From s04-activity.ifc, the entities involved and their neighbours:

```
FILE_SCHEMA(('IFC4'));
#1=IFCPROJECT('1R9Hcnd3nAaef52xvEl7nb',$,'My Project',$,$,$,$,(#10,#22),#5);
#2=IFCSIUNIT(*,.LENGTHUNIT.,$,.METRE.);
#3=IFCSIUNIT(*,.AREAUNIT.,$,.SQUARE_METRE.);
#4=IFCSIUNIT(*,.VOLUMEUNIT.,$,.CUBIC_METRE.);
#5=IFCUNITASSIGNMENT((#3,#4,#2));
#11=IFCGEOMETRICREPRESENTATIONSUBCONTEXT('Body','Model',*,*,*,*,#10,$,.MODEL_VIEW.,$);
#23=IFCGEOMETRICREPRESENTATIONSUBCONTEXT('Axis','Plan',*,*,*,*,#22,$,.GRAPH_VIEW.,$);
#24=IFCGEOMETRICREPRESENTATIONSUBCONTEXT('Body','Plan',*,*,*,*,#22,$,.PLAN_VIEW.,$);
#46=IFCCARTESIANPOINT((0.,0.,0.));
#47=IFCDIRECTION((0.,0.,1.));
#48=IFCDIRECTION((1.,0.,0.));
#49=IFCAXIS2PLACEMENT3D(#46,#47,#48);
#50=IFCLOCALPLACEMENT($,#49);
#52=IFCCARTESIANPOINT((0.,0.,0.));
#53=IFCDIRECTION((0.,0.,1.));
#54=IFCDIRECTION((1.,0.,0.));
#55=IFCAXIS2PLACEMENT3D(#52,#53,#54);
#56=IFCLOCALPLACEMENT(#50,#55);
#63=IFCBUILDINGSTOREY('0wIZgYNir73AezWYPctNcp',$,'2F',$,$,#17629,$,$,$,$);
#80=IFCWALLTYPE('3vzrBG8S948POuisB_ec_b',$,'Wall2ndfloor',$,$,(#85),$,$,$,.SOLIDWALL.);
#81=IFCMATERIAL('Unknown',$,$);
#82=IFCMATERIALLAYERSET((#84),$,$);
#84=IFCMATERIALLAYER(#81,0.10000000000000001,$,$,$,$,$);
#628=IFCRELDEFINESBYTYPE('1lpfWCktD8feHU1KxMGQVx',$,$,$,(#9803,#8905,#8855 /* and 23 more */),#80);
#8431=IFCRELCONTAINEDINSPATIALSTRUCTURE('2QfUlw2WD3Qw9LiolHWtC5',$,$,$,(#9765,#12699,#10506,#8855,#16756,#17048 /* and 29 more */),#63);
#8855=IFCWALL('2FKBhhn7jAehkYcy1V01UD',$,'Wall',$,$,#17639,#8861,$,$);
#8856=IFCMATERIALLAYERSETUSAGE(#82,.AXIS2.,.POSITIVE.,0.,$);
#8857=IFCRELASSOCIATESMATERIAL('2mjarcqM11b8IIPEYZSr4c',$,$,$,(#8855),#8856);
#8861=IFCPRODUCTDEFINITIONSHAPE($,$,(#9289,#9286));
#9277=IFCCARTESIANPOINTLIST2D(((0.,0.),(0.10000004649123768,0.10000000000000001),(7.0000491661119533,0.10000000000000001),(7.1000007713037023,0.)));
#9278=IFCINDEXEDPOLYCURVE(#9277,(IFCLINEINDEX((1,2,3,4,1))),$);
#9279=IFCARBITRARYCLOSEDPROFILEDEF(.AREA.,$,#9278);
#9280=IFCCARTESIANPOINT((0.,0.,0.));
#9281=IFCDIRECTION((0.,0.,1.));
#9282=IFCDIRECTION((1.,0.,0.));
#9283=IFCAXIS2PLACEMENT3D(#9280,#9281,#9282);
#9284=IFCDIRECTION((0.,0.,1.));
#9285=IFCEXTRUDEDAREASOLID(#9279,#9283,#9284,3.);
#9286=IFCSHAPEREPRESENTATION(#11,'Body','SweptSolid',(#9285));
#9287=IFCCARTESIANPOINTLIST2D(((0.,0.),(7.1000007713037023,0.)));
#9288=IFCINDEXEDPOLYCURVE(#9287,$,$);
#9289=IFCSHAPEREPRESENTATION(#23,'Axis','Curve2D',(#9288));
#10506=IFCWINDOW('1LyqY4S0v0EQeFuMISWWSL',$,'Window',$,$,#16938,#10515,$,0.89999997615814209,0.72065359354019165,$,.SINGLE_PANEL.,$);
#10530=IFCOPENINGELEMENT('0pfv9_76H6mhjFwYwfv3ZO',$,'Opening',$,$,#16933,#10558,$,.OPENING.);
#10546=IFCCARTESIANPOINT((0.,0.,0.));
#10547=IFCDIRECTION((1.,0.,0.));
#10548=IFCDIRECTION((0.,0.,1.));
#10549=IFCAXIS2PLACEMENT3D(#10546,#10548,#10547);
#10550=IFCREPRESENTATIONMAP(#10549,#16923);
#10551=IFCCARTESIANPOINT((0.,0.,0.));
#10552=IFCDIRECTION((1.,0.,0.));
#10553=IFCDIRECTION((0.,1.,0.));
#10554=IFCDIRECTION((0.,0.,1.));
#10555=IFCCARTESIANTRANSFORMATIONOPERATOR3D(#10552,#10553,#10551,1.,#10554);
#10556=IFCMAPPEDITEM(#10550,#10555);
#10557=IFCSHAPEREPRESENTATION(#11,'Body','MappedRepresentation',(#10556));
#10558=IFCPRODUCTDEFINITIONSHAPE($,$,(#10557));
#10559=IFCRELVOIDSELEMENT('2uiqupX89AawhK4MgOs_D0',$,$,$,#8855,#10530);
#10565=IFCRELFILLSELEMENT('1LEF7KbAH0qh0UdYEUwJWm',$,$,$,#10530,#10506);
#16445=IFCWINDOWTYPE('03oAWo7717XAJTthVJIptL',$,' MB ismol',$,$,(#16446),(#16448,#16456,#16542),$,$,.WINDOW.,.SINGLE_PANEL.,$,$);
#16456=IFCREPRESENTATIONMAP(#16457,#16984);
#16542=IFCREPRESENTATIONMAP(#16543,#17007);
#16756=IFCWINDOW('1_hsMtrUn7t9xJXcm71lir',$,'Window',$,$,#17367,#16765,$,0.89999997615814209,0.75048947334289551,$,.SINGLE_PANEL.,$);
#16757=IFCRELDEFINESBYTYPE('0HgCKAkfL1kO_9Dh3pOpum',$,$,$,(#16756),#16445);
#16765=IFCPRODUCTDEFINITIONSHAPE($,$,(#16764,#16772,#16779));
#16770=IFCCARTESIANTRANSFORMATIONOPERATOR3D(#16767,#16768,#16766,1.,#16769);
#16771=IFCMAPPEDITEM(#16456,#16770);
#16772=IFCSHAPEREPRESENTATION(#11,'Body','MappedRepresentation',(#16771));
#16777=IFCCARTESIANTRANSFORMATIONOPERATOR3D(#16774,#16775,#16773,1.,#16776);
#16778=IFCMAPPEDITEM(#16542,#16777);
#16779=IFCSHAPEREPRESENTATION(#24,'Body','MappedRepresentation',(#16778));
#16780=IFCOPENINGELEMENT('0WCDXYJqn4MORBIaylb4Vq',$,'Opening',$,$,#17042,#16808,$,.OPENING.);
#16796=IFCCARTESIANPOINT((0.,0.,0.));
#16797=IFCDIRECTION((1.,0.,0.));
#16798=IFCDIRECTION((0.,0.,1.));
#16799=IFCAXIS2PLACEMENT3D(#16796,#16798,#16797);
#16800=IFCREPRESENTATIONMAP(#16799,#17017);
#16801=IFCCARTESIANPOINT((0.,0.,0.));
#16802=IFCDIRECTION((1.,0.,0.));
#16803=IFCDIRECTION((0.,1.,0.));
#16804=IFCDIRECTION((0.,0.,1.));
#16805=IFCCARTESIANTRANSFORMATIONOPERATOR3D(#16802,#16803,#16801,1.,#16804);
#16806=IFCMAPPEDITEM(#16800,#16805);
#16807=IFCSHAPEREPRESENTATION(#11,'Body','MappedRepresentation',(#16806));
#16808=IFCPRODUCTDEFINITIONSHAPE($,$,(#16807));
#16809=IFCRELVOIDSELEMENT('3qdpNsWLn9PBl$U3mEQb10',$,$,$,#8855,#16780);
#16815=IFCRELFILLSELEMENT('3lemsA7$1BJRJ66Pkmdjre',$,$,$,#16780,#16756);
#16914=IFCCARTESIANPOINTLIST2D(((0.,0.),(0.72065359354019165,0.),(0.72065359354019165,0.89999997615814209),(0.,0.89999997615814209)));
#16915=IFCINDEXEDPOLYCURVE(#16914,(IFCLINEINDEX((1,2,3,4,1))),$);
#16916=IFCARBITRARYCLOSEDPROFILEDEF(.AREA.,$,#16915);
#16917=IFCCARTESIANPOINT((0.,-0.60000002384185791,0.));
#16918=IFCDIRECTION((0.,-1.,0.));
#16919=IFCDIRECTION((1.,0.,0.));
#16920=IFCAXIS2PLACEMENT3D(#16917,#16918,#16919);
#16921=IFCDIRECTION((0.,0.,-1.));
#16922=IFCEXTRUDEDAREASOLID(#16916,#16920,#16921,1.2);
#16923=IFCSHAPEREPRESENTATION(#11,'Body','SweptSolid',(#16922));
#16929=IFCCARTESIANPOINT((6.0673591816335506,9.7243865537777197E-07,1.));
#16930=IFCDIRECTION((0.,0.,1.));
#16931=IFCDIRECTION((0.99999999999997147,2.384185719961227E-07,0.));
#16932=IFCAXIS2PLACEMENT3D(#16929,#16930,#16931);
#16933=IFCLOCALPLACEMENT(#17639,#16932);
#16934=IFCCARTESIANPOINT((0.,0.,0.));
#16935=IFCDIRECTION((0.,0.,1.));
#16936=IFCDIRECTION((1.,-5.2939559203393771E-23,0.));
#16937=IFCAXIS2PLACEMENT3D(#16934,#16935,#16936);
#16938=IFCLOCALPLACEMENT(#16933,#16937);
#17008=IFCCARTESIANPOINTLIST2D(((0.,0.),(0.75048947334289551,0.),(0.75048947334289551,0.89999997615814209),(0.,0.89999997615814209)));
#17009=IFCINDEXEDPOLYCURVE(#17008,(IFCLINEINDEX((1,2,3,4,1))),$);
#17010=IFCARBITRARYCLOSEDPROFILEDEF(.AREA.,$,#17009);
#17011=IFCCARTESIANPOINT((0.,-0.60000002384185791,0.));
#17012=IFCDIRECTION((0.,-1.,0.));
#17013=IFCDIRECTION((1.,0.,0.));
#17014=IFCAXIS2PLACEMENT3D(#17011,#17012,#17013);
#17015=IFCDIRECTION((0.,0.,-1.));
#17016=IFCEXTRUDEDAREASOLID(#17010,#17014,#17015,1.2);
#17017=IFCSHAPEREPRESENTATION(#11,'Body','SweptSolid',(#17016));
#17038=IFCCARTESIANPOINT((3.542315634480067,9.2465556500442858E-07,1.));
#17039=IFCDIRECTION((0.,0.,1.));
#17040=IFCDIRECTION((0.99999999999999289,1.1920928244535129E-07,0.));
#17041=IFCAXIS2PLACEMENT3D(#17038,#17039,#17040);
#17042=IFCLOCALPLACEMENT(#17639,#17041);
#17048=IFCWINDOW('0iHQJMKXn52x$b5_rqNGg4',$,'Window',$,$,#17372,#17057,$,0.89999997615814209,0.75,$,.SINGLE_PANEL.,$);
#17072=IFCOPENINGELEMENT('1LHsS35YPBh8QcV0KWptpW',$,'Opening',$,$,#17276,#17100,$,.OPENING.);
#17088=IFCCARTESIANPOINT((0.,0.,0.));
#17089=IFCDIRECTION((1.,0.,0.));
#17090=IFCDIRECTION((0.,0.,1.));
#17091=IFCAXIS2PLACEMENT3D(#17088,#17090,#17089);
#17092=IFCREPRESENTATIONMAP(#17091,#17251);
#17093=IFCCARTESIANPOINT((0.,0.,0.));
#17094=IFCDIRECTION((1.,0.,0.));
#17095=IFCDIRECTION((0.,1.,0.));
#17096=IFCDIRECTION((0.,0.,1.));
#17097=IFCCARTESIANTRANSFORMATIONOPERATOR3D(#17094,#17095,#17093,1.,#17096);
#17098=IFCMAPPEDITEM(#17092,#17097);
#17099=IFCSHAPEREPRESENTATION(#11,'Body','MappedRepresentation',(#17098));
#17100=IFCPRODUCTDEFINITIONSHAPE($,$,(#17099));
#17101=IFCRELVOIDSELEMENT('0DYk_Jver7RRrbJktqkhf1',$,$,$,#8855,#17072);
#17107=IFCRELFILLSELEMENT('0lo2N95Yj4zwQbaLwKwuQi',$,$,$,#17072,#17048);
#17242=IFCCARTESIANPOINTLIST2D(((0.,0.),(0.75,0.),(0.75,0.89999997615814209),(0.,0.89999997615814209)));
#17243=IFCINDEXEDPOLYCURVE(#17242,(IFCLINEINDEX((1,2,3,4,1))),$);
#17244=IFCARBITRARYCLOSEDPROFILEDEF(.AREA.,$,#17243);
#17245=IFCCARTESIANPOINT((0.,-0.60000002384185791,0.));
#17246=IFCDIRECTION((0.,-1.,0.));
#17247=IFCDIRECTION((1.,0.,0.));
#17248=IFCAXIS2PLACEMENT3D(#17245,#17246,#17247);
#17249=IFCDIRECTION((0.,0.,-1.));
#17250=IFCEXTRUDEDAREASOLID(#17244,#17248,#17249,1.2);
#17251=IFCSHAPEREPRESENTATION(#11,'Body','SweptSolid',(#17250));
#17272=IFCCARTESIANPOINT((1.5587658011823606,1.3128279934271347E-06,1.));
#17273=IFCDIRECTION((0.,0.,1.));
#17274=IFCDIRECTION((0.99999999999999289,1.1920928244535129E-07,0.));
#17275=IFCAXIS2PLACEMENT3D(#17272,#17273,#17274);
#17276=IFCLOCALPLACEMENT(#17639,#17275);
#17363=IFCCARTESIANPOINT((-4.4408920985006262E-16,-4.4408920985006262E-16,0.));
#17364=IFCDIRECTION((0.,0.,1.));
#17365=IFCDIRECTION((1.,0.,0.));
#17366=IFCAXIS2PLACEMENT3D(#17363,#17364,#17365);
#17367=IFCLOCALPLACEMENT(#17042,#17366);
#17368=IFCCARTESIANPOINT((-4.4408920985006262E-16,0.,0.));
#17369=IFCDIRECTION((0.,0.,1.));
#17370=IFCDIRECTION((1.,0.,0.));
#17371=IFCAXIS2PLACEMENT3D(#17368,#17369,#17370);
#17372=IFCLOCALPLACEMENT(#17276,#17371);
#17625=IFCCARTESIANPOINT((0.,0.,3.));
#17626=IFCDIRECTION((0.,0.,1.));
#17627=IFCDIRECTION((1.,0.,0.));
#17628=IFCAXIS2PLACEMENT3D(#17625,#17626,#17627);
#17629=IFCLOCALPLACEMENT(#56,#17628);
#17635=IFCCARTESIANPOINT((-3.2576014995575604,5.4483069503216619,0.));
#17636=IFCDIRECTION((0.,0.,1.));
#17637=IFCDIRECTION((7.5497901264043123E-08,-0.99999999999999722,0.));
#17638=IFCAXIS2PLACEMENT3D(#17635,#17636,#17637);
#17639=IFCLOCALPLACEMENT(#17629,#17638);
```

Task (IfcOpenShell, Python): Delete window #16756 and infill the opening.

```python
import ifcopenshell
import ifcopenshell.api.feature
import ifcopenshell.api.root
import ifcopenshell.geom
import ifcopenshell.util.shape

model = ifcopenshell.open("s04-activity.ifc")
settings = ifcopenshell.geom.settings()


def volume(element):
    """Net volume in cubic metres, openings subtracted."""
    shape = ifcopenshell.geom.create_shape(settings, element)
    return ifcopenshell.util.shape.get_volume(shape.geometry)


window = model.by_guid("1_hsMtrUn7t9xJXcm71lir")
opening = window.FillsVoids[0].RelatingOpeningElement
wall = opening.VoidsElements[0].RelatingBuildingElement
before = volume(wall)

ifcopenshell.api.root.remove_product(model, product=window)
ifcopenshell.api.feature.remove_feature(model, feature=opening)

after = volume(wall)

print(f"wall volume {before:.3f} -> {after:.3f} m3")

model.write("s04-activity_edited.ifc")
```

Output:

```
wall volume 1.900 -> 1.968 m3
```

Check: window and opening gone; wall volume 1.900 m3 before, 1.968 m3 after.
